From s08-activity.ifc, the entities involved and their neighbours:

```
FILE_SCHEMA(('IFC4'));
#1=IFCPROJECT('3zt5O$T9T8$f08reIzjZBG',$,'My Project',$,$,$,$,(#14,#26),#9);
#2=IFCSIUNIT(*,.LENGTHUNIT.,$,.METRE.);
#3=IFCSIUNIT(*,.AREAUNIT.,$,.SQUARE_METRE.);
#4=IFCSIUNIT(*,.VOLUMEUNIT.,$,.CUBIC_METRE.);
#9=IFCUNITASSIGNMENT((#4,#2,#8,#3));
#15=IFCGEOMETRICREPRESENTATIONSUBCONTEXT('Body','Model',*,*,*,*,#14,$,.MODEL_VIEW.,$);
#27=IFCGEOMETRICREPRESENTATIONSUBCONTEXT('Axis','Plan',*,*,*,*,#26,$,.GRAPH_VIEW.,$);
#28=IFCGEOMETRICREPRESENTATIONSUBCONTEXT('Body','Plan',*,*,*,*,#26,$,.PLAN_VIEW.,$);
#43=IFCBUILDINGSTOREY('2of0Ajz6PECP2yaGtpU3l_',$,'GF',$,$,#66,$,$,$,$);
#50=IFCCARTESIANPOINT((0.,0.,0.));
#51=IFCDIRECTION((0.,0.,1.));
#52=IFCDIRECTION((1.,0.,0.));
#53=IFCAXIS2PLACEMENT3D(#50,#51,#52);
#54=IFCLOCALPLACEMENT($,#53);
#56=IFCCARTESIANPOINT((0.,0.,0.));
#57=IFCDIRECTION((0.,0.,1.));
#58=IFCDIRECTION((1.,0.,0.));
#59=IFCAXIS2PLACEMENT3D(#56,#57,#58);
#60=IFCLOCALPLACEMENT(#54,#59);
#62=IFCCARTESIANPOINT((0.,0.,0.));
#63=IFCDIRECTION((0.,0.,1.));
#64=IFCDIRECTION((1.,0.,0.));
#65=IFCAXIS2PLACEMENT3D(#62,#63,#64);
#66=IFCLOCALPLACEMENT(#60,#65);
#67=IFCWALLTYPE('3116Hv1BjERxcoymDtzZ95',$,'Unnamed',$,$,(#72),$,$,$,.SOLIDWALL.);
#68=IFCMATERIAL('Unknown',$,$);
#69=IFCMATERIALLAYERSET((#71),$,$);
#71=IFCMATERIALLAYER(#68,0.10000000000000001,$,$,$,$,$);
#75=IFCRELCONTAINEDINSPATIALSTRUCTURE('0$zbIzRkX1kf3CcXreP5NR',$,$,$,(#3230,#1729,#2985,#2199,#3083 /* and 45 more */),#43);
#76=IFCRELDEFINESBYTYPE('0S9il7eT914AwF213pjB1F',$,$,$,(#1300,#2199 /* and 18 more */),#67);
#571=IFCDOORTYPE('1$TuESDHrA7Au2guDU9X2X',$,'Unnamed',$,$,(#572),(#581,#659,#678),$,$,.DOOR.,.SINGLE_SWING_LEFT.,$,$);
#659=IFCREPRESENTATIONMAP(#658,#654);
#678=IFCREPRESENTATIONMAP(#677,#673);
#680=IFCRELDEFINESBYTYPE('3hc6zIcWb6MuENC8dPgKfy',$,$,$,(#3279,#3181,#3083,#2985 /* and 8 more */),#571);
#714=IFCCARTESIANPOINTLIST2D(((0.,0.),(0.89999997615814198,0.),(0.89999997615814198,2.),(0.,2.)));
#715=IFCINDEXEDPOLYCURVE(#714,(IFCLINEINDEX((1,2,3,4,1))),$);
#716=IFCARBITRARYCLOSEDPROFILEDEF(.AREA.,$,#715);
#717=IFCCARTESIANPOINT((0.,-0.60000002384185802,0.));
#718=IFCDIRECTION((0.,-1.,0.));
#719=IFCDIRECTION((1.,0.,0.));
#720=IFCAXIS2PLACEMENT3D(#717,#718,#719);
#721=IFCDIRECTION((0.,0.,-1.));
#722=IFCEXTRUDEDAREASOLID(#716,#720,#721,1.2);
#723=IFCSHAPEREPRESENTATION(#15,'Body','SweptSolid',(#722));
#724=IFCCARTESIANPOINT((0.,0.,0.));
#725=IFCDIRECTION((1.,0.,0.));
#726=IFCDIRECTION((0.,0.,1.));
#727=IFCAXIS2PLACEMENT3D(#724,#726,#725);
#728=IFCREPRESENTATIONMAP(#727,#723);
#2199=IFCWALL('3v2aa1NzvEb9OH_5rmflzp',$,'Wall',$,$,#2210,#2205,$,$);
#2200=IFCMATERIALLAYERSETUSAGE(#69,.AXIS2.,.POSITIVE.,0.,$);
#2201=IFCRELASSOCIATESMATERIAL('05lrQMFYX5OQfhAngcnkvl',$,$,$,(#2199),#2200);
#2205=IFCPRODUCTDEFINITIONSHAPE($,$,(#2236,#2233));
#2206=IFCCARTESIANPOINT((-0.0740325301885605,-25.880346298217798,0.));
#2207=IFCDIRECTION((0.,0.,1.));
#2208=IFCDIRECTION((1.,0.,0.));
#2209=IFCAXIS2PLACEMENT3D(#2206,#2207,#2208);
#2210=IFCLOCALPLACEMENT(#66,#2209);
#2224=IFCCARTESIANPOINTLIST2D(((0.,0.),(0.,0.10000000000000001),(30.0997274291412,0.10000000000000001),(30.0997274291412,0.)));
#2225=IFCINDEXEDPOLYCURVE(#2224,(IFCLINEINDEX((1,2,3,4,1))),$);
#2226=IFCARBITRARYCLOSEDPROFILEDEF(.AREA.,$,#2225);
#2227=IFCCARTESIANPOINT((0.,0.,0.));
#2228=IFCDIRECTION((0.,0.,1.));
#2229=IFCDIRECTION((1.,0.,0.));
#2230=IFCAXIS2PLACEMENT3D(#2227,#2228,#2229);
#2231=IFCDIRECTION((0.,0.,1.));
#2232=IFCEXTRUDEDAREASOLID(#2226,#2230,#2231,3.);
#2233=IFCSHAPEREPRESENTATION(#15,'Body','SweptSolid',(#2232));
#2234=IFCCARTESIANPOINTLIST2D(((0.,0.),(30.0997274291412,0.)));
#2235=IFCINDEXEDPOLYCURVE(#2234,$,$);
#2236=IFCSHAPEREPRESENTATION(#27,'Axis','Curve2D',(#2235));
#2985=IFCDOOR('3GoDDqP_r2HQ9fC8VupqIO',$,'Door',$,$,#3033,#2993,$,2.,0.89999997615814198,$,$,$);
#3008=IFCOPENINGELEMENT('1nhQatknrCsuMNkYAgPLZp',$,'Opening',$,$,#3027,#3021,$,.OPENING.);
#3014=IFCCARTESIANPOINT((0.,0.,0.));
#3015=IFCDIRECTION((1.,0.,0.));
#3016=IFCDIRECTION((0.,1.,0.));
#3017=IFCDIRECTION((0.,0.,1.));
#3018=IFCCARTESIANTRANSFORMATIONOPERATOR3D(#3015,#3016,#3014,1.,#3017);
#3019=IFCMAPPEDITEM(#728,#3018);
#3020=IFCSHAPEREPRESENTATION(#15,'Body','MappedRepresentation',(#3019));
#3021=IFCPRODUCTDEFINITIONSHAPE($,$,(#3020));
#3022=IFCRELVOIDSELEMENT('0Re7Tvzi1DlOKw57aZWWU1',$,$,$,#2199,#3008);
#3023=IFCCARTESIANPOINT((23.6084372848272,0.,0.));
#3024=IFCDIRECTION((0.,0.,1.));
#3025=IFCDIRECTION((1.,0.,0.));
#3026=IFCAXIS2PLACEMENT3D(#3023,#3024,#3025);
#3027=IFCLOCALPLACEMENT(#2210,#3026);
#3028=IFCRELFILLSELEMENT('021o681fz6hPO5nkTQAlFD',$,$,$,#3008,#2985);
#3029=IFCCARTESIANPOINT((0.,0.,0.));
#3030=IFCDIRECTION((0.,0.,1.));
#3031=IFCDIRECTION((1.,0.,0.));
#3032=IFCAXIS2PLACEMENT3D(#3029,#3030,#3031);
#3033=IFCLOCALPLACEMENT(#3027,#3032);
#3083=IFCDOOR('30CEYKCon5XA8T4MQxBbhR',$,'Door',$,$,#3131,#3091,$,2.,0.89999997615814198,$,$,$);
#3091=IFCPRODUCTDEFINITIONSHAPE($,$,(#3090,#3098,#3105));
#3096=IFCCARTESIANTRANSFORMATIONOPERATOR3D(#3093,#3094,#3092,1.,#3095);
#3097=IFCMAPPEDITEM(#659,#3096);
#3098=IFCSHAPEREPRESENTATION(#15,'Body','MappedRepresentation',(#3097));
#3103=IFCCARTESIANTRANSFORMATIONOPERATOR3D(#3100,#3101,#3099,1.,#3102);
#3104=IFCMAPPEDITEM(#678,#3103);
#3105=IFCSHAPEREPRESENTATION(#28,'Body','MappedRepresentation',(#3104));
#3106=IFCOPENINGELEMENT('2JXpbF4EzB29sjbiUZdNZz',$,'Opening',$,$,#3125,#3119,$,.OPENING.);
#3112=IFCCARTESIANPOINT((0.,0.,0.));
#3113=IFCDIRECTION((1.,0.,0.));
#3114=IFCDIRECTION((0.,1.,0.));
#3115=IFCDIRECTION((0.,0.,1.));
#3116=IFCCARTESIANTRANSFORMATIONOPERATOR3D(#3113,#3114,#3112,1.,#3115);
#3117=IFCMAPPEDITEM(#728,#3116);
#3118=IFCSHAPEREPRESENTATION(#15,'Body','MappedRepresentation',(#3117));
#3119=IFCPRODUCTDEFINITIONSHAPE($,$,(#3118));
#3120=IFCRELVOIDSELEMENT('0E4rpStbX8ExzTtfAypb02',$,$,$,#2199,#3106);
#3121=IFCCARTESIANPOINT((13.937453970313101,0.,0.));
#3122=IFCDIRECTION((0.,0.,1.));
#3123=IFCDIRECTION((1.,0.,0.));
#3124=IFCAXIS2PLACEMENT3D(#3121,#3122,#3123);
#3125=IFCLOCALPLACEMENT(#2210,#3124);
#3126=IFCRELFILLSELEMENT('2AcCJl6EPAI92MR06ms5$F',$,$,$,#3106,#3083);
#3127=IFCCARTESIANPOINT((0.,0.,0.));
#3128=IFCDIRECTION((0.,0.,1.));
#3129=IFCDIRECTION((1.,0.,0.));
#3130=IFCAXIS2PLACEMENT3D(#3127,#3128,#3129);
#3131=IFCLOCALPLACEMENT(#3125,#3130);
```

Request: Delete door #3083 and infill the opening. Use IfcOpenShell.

```python
import ifcopenshell
import ifcopenshell.api.feature
import ifcopenshell.api.root
import ifcopenshell.geom
import ifcopenshell.util.shape

model = ifcopenshell.open("s08-activity.ifc")
settings = ifcopenshell.geom.settings()


def volume(element):
    """Net volume in cubic metres, openings subtracted."""
    shape = ifcopenshell.geom.create_shape(settings, element)
    return ifcopenshell.util.shape.get_volume(shape.geometry)


door = model.by_guid("30CEYKCon5XA8T4MQxBbhR")
opening = door.FillsVoids[0].RelatingOpeningElement
wall = opening.VoidsElements[0].RelatingBuildingElement
before = volume(wall)

ifcopenshell.api.root.remove_product(model, product=door)
ifcopenshell.api.feature.remove_feature(model, feature=opening)

after = volume(wall)

print(f"wall volume {before:.3f} -> {after:.3f} m3")

model.write("s08-activity_rev.ifc")
```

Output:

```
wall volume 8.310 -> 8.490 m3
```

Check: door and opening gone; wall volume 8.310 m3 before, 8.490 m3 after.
